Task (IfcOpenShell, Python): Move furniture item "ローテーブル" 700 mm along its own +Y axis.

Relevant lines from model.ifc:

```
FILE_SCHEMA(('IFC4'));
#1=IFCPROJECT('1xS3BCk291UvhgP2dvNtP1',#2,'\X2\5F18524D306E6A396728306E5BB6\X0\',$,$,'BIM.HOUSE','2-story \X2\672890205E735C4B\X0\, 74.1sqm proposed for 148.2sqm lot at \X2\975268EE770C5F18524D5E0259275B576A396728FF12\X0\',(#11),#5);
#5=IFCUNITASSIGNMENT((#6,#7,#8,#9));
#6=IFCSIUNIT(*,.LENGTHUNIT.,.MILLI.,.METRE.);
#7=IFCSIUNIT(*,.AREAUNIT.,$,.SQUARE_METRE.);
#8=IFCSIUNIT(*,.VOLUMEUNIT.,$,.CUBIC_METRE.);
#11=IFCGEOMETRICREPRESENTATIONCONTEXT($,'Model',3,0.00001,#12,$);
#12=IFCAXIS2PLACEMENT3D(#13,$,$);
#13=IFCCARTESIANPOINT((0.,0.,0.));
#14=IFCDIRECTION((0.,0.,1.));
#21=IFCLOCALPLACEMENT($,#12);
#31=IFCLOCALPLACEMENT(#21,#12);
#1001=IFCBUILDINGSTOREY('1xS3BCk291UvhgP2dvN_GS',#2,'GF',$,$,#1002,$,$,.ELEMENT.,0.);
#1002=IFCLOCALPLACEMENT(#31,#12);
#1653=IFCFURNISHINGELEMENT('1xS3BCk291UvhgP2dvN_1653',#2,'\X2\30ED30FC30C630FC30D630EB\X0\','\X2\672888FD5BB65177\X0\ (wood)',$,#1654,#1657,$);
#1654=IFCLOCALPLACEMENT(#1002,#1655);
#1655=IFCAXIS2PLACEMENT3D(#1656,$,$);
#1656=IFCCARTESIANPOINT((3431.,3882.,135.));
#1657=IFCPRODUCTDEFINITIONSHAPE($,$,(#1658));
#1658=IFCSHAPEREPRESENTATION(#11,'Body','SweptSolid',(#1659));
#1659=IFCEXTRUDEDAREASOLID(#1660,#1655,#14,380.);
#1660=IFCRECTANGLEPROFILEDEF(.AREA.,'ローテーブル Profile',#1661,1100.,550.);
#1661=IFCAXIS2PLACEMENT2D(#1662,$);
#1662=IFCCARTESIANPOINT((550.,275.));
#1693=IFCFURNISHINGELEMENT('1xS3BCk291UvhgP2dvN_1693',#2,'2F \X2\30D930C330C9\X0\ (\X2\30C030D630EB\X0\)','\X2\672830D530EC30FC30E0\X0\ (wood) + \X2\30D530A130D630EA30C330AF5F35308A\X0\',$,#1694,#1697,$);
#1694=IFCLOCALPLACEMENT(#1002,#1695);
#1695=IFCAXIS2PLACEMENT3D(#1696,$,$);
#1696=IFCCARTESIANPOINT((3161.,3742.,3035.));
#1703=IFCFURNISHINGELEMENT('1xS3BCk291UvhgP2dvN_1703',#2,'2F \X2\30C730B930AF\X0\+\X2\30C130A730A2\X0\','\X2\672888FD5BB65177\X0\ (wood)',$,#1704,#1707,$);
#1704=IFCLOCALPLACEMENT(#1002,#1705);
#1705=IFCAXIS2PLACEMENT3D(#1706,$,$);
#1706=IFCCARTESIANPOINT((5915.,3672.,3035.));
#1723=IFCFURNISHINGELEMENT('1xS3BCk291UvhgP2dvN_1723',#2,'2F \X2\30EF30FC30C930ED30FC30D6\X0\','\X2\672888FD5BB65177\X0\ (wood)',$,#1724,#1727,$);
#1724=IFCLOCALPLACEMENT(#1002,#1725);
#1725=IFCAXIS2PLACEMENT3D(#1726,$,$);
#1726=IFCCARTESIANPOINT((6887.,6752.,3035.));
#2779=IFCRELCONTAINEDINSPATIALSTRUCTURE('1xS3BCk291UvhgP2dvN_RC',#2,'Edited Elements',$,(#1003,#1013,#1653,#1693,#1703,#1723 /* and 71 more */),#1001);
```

```python
import ifcopenshell
import ifcopenshell.api.geometry
import ifcopenshell.util.placement
import ifcopenshell.util.unit

model = ifcopenshell.open("model.ifc")
unit_scale = ifcopenshell.util.unit.calculate_unit_scale(model)

item = model.by_guid("1xS3BCk291UvhgP2dvN_1653")
matrix = ifcopenshell.util.placement.get_local_placement(item.ObjectPlacement)
matrix[:3, 3] += matrix[:3, 1] * 0.7 / unit_scale
ifcopenshell.api.geometry.edit_object_placement(model, product=item, matrix=matrix, is_si=False)

print(ifcopenshell.util.placement.get_local_placement(item.ObjectPlacement).round(3) + 0.0)

model.write("model_v2.ifc")
```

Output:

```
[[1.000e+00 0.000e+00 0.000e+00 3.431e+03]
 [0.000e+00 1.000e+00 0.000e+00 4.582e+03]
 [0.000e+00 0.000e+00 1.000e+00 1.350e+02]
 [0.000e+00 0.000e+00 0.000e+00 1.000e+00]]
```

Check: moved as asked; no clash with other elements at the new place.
